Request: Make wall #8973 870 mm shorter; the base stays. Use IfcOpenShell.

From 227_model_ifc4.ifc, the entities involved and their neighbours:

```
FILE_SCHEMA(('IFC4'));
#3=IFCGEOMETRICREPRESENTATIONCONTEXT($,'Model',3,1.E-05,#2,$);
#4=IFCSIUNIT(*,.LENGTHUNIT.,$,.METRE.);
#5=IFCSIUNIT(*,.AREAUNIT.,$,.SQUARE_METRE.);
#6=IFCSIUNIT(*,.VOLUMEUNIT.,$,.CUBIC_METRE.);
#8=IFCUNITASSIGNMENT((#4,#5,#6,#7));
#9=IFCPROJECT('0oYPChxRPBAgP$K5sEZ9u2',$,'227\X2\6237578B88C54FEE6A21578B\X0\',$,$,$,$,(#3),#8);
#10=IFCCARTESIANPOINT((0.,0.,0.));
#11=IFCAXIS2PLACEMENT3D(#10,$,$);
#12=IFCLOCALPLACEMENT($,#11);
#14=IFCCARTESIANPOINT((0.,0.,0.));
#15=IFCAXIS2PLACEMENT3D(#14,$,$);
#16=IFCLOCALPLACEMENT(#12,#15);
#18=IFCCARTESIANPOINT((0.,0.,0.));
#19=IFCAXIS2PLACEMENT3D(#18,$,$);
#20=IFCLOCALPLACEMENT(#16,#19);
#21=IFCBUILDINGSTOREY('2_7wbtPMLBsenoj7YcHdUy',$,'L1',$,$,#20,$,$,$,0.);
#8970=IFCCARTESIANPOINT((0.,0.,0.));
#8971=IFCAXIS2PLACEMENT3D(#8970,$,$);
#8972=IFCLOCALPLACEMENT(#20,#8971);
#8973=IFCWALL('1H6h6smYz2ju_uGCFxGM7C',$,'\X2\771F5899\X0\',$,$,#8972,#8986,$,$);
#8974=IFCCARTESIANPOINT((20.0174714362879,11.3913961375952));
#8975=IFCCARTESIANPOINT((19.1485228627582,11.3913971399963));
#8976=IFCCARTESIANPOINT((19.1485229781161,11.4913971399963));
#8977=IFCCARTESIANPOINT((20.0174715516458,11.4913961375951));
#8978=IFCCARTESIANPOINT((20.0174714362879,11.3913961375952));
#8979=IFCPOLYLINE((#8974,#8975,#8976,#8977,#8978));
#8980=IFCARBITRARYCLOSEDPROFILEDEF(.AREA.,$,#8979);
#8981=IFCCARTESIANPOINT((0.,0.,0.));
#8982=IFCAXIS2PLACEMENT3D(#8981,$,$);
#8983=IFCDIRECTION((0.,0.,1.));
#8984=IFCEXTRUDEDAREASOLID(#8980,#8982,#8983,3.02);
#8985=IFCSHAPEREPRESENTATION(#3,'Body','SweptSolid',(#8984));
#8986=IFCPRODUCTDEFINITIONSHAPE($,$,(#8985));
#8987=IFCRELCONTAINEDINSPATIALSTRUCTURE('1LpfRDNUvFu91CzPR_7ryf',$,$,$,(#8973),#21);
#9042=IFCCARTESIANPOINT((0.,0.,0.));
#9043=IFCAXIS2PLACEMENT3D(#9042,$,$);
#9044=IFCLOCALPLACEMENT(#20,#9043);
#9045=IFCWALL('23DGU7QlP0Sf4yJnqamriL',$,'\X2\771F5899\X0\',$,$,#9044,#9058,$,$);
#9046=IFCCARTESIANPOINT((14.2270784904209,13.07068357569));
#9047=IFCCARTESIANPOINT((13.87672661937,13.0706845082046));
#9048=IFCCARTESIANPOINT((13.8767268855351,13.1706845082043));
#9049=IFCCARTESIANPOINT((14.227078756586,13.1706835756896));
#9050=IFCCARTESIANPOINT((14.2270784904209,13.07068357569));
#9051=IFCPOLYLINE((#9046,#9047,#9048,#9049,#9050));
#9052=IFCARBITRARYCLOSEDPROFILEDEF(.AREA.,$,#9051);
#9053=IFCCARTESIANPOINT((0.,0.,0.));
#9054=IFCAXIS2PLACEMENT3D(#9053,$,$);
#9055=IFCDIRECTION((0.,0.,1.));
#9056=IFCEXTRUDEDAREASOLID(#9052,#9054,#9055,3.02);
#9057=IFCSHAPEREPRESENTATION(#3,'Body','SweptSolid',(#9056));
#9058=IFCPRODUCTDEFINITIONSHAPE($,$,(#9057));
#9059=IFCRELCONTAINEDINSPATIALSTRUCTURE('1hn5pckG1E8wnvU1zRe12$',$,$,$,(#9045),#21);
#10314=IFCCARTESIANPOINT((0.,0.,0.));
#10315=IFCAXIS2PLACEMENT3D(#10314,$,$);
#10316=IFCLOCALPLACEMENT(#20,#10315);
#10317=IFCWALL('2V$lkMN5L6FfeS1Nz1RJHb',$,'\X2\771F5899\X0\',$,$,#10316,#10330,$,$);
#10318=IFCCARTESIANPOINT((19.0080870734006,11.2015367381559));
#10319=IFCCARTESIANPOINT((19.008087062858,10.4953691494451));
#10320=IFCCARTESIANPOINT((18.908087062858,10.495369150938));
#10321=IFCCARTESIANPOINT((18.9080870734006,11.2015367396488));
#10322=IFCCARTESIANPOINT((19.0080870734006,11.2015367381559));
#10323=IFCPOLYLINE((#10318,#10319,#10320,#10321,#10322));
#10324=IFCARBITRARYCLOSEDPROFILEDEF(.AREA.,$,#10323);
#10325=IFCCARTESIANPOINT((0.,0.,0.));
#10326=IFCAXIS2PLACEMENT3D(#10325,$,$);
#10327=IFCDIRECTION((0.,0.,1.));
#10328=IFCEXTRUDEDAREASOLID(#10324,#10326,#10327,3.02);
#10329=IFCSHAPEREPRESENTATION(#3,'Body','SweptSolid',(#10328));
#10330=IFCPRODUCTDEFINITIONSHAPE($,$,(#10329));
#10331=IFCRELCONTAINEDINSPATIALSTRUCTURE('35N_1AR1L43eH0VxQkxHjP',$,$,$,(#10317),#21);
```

```python
import ifcopenshell
import ifcopenshell.geom
import ifcopenshell.util.shape

model = ifcopenshell.open("227_model_ifc4.ifc")
settings = ifcopenshell.geom.settings()


def volume(element):
    """Net volume in cubic metres, openings subtracted."""
    shape = ifcopenshell.geom.create_shape(settings, element)
    return ifcopenshell.util.shape.get_volume(shape.geometry)


wall = model.by_id(8973)
before = volume(wall)

body = next(r for r in wall.Representation.Representations if r.RepresentationIdentifier == "Body")
solid = body.Items[0]
old_height = solid.Depth
solid.Depth -= 0.87
after = volume(wall)

print(f"height {old_height:g} -> {solid.Depth:g}, volume {before:.3f} -> {after:.3f} m3")

model.write("227_model_ifc4-out.ifc")
```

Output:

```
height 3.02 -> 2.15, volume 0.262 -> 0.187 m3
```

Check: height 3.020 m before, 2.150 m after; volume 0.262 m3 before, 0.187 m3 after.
